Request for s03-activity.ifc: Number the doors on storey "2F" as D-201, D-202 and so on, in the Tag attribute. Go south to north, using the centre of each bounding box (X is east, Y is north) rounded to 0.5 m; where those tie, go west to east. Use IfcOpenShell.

First a look at what the model holds.

```python
import ifcopenshell
import ifcopenshell.util.element
import ifcopenshell.util.placement

model = ifcopenshell.open("s03-activity.ifc")
print(model.schema)
storey = next(s for s in model.by_type("IfcBuildingStorey") if s.Name == "2F")
doors = [e for e in ifcopenshell.util.element.get_decomposition(storey) if e.is_a("IfcDoor")]
for e in sorted(doors, key=lambda e: e.id()):
    origin = ifcopenshell.util.placement.get_local_placement(e.ObjectPlacement)[:3, 3]
    print(e.id(), e.Tag, e.Name, origin.round(2) + 0.0, sep=" | ")
```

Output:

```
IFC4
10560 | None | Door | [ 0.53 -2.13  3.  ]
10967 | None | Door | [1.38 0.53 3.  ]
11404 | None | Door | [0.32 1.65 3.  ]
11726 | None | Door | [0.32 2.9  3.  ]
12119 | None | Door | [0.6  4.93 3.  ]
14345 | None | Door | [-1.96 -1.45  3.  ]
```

```python
import ifcopenshell
import ifcopenshell.geom
import ifcopenshell.util.element
import ifcopenshell.util.shape

model = ifcopenshell.open("s03-activity.ifc")
settings = ifcopenshell.geom.settings()
settings.set("use-world-coords", True)


def centre(element):
    shape = ifcopenshell.geom.create_shape(settings, element)
    return ifcopenshell.util.shape.get_bbox_centroid(shape.geometry)


storey = next(s for s in model.by_type("IfcBuildingStorey") if s.Name == "2F")
doors = [e for e in ifcopenshell.util.element.get_decomposition(storey) if e.is_a("IfcDoor")]

# Insertion points can sit at a corner or the storey origin, so sort by the geometry (in metres).
centres = {e: centre(e) for e in doors}
doors.sort(key=lambda e: (round(centres[e][1] / 0.5), centres[e][0]))

for i, e in enumerate(doors, start=1):
    number = f"D-2{i:02d}"
    e.Tag = number
    print(e.id(), number)

model.write("s03-activity_updated.ifc")
```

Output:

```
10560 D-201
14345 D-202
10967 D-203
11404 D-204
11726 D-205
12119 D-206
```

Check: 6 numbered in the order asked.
